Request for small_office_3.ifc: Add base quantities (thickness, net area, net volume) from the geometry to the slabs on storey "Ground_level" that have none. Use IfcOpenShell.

First a look at what the model holds.

```python
import ifcopenshell
import ifcopenshell.util.element
import ifcopenshell.util.unit

model = ifcopenshell.open("small_office_3.ifc")
print(model.schema)
for unit_type in ("LENGTHUNIT", "AREAUNIT", "VOLUMEUNIT"):
    print(unit_type, ifcopenshell.util.unit.calculate_unit_scale(model, unit_type))
storey = next(s for s in model.by_type("IfcBuildingStorey") if s.Name == "Ground_level")
slabs = [e for e in ifcopenshell.util.element.get_decomposition(storey) if e.is_a("IfcSlab")]
for e in sorted(slabs, key=lambda e: e.id()):
    print(e.id(), e.is_a(), e.Name, list(ifcopenshell.util.element.get_psets(e, qtos_only=True)), sep=" | ")
```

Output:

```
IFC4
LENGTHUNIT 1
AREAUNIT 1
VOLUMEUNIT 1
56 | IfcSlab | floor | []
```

```python
import ifcopenshell
import ifcopenshell.api.pset
import ifcopenshell.geom
import ifcopenshell.util.element
import ifcopenshell.util.shape
import ifcopenshell.util.unit

model = ifcopenshell.open("small_office_3.ifc")
unit_scale = ifcopenshell.util.unit.calculate_unit_scale(model)
area_scale = ifcopenshell.util.unit.calculate_unit_scale(model, "AREAUNIT")
volume_scale = ifcopenshell.util.unit.calculate_unit_scale(model, "VOLUMEUNIT")
settings = ifcopenshell.geom.settings()

storey = next(s for s in model.by_type("IfcBuildingStorey") if s.Name == "Ground_level")
slabs = [e for e in ifcopenshell.util.element.get_decomposition(storey) if e.is_a("IfcSlab")]

for e in sorted(slabs, key=lambda e: e.id()):
    if ifcopenshell.util.element.get_psets(e, qtos_only=True, should_inherit=False):
        continue
    # Geometry comes back in metres, in the element's own axes.
    shape = ifcopenshell.geom.create_shape(settings, e)
    values = {
        "Width": ifcopenshell.util.shape.get_z(shape.geometry) / unit_scale,
        "NetArea": ifcopenshell.util.shape.get_footprint_area(shape.geometry) / area_scale,
        "NetVolume": ifcopenshell.util.shape.get_volume(shape.geometry) / volume_scale,
    }
    qto = ifcopenshell.api.pset.add_qto(model, product=e, name="Qto_SlabBaseQuantities")
    ifcopenshell.api.pset.edit_qto(model, qto=qto, properties=values)
    print(e.id(), {k: round(v, 3) for k, v in values.items()})

model.write("small_office_3_edited.ifc")
```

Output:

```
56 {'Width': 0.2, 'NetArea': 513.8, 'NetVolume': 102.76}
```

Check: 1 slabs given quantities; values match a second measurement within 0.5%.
